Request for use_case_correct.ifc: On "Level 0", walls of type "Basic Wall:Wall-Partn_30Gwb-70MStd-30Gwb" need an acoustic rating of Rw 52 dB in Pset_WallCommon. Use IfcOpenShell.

First a look at what the model holds.

```python
import ifcopenshell
import ifcopenshell.util.element

model = ifcopenshell.open("use_case_correct.ifc")
print(model.schema)
storey = next(s for s in model.by_type("IfcBuildingStorey") if s.Name == "Level 0")
walls = [e for e in ifcopenshell.util.element.get_decomposition(storey) if e.is_a("IfcWall")]
seen = {}
for e in walls:
    element_type = ifcopenshell.util.element.get_type(e)
    key = (element_type.Name if element_type != e and element_type else None, ifcopenshell.util.element.get_pset(e, "Pset_WallCommon", "AcousticRating"))
    seen[key] = seen.get(key, 0) + 1
for (name, value), count in sorted(seen.items(), key=str):
    print(count, "x", name, "|", value)
```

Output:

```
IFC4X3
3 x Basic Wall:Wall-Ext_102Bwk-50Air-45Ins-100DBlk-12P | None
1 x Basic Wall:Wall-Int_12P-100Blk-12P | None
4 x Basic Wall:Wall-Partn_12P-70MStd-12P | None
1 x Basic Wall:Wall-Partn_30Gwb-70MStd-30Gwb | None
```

```python
import ifcopenshell
import ifcopenshell.api.pset
import ifcopenshell.util.element

model = ifcopenshell.open("use_case_correct.ifc")

storey = next(s for s in model.by_type("IfcBuildingStorey") if s.Name == "Level 0")
walls = [e for e in ifcopenshell.util.element.get_decomposition(storey) if e.is_a("IfcWall")]

count = 0
for e in walls:
    element_type = ifcopenshell.util.element.get_type(e)
    if element_type in (None, e) or element_type.Name != "Basic Wall:Wall-Partn_30Gwb-70MStd-30Gwb":
        continue
    # add_pset returns the element's existing set when there is one.
    pset = ifcopenshell.api.pset.add_pset(model, product=e, name="Pset_WallCommon")
    ifcopenshell.api.pset.edit_pset(model, pset=pset, properties={"AcousticRating": "Rw 52 dB"})
    count += 1

print(count, "walls updated")

model.write("use_case_correct_rev.ifc")
```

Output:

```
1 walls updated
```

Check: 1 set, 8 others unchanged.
